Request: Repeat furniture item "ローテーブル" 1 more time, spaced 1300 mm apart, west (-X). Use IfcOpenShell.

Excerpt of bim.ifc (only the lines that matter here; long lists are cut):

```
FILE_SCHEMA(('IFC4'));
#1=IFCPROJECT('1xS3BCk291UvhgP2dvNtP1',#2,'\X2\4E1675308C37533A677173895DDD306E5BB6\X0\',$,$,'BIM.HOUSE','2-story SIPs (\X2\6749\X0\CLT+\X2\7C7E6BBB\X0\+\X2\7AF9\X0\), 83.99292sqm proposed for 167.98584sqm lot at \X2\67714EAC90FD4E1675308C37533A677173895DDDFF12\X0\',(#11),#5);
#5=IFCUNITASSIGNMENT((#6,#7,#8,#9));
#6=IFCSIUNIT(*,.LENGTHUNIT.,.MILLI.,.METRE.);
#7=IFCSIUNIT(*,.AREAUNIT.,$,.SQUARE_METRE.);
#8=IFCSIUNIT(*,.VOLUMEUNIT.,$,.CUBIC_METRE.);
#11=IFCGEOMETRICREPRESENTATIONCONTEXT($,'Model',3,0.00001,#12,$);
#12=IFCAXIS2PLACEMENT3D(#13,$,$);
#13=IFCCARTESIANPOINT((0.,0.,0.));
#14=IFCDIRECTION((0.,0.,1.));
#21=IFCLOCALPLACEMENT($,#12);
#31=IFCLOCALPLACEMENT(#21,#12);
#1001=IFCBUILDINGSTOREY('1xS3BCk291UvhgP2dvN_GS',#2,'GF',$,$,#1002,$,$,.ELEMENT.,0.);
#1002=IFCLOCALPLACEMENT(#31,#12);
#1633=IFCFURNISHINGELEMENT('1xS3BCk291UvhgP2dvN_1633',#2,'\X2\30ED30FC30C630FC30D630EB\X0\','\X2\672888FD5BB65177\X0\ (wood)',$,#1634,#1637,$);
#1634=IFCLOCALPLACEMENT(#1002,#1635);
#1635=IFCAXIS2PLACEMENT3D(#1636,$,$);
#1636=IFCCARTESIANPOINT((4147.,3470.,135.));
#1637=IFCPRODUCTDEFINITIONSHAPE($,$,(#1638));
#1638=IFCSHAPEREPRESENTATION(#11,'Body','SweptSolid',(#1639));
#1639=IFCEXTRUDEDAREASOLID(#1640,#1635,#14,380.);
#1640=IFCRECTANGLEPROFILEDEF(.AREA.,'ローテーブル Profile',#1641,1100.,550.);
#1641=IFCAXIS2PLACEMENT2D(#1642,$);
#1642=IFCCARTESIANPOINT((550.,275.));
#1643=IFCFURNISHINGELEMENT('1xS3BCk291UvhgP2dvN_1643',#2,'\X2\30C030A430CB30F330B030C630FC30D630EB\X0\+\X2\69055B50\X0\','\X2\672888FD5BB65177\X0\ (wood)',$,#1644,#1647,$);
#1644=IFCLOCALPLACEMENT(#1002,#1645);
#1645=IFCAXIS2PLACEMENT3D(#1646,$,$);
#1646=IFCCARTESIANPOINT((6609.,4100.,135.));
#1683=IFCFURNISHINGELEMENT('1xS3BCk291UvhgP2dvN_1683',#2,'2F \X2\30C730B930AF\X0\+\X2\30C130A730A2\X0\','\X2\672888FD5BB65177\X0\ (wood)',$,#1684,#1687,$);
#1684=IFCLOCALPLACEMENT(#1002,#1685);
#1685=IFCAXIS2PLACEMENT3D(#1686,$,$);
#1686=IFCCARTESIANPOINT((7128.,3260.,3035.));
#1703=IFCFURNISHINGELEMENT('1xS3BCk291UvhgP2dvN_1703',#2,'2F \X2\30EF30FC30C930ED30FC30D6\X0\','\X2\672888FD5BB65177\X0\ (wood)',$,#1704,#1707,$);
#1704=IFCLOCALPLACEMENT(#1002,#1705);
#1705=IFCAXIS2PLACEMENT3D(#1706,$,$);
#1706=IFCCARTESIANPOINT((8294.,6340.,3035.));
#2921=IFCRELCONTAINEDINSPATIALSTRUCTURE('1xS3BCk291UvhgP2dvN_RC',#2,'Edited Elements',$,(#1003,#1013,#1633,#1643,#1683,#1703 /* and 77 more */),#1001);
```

```python
import numpy as np
import ifcopenshell
import ifcopenshell.api.geometry
import ifcopenshell.api.root
import ifcopenshell.util.element
import ifcopenshell.util.placement
import ifcopenshell.util.unit

model = ifcopenshell.open("bim.ifc")
unit_scale = ifcopenshell.util.unit.calculate_unit_scale(model)


def reuse_history(source, copy):
    """copy_class also copies each property set's owner history, people and application; keep the originals."""
    for rel in copy.IsDefinedBy:
        if rel.is_a("IfcRelDefinesByProperties") and (history := rel.RelatingPropertyDefinition.OwnerHistory):
            rel.RelatingPropertyDefinition.OwnerHistory = source.OwnerHistory
            ifcopenshell.util.element.remove_deep2(model, history)


source = model.by_guid("1xS3BCk291UvhgP2dvN_1633")
base = ifcopenshell.util.placement.get_local_placement(source.ObjectPlacement)
step = np.array([-1.0, 0.0, 0.0]) * 1.3 / unit_scale

for i in range(1, 2):
    copy = ifcopenshell.api.root.copy_class(model, product=source)
    copy.Representation = ifcopenshell.util.element.copy_deep(
        model, source.Representation, exclude=["IfcGeometricRepresentationContext", "IfcRepresentationMap"]
    )
    reuse_history(source, copy)
    matrix = base.copy()
    matrix[:3, 3] += i * step
    print("added at", matrix[:3, 3].round(3) + 0.0)
    ifcopenshell.api.geometry.edit_object_placement(model, product=copy, matrix=matrix, is_si=False)

model.write("bim_v2.ifc")
```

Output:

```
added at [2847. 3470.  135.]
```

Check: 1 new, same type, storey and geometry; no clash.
